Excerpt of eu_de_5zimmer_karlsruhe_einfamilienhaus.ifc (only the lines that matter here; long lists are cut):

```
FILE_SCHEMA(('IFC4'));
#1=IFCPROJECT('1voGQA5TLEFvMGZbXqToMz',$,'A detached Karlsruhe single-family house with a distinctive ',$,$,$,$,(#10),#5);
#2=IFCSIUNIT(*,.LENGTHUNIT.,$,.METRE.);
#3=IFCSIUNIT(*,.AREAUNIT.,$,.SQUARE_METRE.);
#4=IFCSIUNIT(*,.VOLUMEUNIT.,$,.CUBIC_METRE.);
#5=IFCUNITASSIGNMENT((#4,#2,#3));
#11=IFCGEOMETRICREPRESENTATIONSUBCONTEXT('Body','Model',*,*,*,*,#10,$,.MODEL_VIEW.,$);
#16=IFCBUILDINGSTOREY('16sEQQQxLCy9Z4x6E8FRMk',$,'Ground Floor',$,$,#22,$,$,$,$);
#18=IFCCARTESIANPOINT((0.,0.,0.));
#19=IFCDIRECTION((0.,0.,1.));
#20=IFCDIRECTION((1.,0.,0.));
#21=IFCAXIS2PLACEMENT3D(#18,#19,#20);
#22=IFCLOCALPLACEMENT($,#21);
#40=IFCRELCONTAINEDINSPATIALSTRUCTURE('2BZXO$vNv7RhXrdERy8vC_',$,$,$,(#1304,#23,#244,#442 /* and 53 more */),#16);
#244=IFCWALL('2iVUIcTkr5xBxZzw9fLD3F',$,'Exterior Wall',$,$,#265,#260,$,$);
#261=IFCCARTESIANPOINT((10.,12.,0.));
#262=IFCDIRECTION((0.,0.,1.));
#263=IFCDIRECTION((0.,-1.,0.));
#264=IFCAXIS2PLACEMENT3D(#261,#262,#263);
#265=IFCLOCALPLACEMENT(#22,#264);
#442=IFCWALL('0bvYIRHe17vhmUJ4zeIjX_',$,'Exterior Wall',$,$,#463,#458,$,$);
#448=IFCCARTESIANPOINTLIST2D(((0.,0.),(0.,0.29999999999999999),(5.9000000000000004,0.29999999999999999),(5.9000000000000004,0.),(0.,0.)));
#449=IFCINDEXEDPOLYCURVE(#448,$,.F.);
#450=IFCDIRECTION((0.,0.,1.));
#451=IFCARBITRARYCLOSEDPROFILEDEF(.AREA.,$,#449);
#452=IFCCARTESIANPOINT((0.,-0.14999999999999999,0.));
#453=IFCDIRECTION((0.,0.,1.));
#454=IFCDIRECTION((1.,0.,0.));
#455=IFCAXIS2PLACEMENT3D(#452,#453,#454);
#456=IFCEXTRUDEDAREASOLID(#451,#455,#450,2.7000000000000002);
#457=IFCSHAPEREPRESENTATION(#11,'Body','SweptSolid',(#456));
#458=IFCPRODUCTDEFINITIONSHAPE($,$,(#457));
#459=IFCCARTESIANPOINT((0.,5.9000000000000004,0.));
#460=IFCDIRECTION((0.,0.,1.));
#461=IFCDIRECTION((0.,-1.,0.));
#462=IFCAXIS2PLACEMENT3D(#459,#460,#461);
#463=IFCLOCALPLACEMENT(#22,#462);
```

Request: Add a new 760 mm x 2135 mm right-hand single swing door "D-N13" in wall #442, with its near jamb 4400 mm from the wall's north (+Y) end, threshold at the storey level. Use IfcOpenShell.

```python
import numpy as np
import ifcopenshell
import ifcopenshell.api.feature
import ifcopenshell.api.geometry
import ifcopenshell.api.root
import ifcopenshell.api.spatial
import ifcopenshell.geom
import ifcopenshell.util.element
import ifcopenshell.util.placement
import ifcopenshell.util.representation
import ifcopenshell.util.shape
import ifcopenshell.util.unit

model = ifcopenshell.open("eu_de_5zimmer_karlsruhe_einfamilienhaus.ifc")
unit_scale = ifcopenshell.util.unit.calculate_unit_scale(model)
settings = ifcopenshell.geom.settings()


def volume(element):
    """Net volume in cubic metres, openings subtracted."""
    shape = ifcopenshell.geom.create_shape(settings, element)
    return ifcopenshell.util.shape.get_volume(shape.geometry)


wall = model.by_id(442)
storey = ifcopenshell.util.element.get_container(wall, ifc_class="IfcBuildingStorey")
context = ifcopenshell.util.representation.get_context(model, "Model", "Body", "MODEL_VIEW")
before = volume(wall)

width, height, from_end, sill = 0.76, 2.135, 4.4, 0.0  # metres

# The wall runs along its own X axis, and the end named is its -X end.
wall_shape = ifcopenshell.geom.create_shape(settings, wall)
x, y, z = ifcopenshell.util.shape.get_vertices(wall_shape.geometry).T
start = x.min() + from_end
face, thickness = float(y.min()), float(y.max() - y.min())
wall_matrix = ifcopenshell.util.placement.get_local_placement(wall.ObjectPlacement)
level = ifcopenshell.util.placement.get_local_placement(storey.ObjectPlacement)[2, 3]


def in_wall(x, y):
    """Placement at x, y metres in the wall's axes, at sill height."""
    matrix = wall_matrix.copy()
    matrix[:, 3] = wall_matrix @ np.array([x / unit_scale, y / unit_scale, 0.0, 1.0])
    matrix[2, 3] = level + sill / unit_scale
    return matrix


# Opening: a box that overshoots both wall faces by 50 mm.
opening = ifcopenshell.api.root.create_entity(model, ifc_class="IfcOpeningElement", predefined_type="OPENING")
box = ifcopenshell.api.geometry.add_wall_representation(
    model, context=context, length=width, height=height, thickness=thickness + 0.1
)
ifcopenshell.api.geometry.assign_representation(model, product=opening, representation=box)
ifcopenshell.api.geometry.edit_object_placement(model, product=opening, matrix=in_wall(start, face - 0.05), is_si=False)
ifcopenshell.api.feature.add_feature(model, feature=opening, element=wall)

door = ifcopenshell.api.root.create_entity(model, ifc_class="IfcDoor", name="D-N13", predefined_type="DOOR")
door.OverallWidth, door.OverallHeight = width / unit_scale, height / unit_scale
door.OperationType = "SINGLE_SWING_RIGHT"
body = ifcopenshell.api.geometry.add_door_representation(
    model,
    context=context,
    overall_width=door.OverallWidth,
    overall_height=door.OverallHeight,
    operation_type="SINGLE_SWING_RIGHT",
    lining_properties={"LiningDepth": thickness / unit_scale, "ThresholdDepth": thickness / unit_scale},
)
ifcopenshell.api.geometry.assign_representation(model, product=door, representation=body)
ifcopenshell.api.spatial.assign_container(model, products=[door], relating_structure=storey)
ifcopenshell.api.feature.add_filling(model, opening=opening, element=door)

# The lining spans the wall, so the door starts at the wall face.
ifcopenshell.api.geometry.edit_object_placement(model, product=door, matrix=in_wall(start, face), is_si=False)

after = volume(wall)

print(f"wall volume {before:.3f} -> {after:.3f} m3")

model.write("eu_de_5zimmer_karlsruhe_einfamilienhaus_edited.ifc")
```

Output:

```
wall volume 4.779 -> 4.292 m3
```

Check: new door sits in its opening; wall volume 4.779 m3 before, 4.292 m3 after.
